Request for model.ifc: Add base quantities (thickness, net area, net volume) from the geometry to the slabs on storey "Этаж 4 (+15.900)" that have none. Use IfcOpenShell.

First a look at what the model holds.

```python
import ifcopenshell
import ifcopenshell.util.element
import ifcopenshell.util.unit

model = ifcopenshell.open("model.ifc")
print(model.schema)
for unit_type in ("LENGTHUNIT", "AREAUNIT", "VOLUMEUNIT"):
    print(unit_type, ifcopenshell.util.unit.calculate_unit_scale(model, unit_type))
storey = next(s for s in model.by_type("IfcBuildingStorey") if s.Name == "Этаж 4 (+15.900)")
slabs = [e for e in ifcopenshell.util.element.get_decomposition(storey) if e.is_a("IfcSlab")]
for e in sorted(slabs, key=lambda e: e.id()):
    print(e.id(), e.is_a(), e.Name, list(ifcopenshell.util.element.get_psets(e, qtos_only=True)), sep=" | ")
```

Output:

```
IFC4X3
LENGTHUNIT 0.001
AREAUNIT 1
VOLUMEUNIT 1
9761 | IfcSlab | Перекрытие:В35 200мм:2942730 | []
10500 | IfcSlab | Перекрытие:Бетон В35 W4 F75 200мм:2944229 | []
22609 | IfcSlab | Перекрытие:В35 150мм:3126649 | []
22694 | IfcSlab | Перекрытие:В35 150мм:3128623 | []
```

```python
import ifcopenshell
import ifcopenshell.api.pset
import ifcopenshell.geom
import ifcopenshell.util.element
import ifcopenshell.util.shape
import ifcopenshell.util.unit

model = ifcopenshell.open("model.ifc")
unit_scale = ifcopenshell.util.unit.calculate_unit_scale(model)
area_scale = ifcopenshell.util.unit.calculate_unit_scale(model, "AREAUNIT")
volume_scale = ifcopenshell.util.unit.calculate_unit_scale(model, "VOLUMEUNIT")
settings = ifcopenshell.geom.settings()

storey = next(s for s in model.by_type("IfcBuildingStorey") if s.Name == "Этаж 4 (+15.900)")
slabs = [e for e in ifcopenshell.util.element.get_decomposition(storey) if e.is_a("IfcSlab")]

for e in sorted(slabs, key=lambda e: e.id()):
    if ifcopenshell.util.element.get_psets(e, qtos_only=True, should_inherit=False):
        continue
    # Geometry comes back in metres, in the element's own axes.
    shape = ifcopenshell.geom.create_shape(settings, e)
    values = {
        "Width": ifcopenshell.util.shape.get_z(shape.geometry) / unit_scale,
        "NetArea": ifcopenshell.util.shape.get_footprint_area(shape.geometry) / area_scale,
        "NetVolume": ifcopenshell.util.shape.get_volume(shape.geometry) / volume_scale,
    }
    qto = ifcopenshell.api.pset.add_qto(model, product=e, name="Qto_SlabBaseQuantities")
    ifcopenshell.api.pset.edit_qto(model, qto=qto, properties=values)
    print(e.id(), {k: round(v, 3) for k, v in values.items()})

model.write("model_rev.ifc")
```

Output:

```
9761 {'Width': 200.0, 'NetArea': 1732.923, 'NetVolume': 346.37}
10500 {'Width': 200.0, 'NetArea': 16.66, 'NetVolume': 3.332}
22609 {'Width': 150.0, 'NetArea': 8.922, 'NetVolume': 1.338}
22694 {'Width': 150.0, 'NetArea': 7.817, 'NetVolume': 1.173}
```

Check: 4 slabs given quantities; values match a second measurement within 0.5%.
